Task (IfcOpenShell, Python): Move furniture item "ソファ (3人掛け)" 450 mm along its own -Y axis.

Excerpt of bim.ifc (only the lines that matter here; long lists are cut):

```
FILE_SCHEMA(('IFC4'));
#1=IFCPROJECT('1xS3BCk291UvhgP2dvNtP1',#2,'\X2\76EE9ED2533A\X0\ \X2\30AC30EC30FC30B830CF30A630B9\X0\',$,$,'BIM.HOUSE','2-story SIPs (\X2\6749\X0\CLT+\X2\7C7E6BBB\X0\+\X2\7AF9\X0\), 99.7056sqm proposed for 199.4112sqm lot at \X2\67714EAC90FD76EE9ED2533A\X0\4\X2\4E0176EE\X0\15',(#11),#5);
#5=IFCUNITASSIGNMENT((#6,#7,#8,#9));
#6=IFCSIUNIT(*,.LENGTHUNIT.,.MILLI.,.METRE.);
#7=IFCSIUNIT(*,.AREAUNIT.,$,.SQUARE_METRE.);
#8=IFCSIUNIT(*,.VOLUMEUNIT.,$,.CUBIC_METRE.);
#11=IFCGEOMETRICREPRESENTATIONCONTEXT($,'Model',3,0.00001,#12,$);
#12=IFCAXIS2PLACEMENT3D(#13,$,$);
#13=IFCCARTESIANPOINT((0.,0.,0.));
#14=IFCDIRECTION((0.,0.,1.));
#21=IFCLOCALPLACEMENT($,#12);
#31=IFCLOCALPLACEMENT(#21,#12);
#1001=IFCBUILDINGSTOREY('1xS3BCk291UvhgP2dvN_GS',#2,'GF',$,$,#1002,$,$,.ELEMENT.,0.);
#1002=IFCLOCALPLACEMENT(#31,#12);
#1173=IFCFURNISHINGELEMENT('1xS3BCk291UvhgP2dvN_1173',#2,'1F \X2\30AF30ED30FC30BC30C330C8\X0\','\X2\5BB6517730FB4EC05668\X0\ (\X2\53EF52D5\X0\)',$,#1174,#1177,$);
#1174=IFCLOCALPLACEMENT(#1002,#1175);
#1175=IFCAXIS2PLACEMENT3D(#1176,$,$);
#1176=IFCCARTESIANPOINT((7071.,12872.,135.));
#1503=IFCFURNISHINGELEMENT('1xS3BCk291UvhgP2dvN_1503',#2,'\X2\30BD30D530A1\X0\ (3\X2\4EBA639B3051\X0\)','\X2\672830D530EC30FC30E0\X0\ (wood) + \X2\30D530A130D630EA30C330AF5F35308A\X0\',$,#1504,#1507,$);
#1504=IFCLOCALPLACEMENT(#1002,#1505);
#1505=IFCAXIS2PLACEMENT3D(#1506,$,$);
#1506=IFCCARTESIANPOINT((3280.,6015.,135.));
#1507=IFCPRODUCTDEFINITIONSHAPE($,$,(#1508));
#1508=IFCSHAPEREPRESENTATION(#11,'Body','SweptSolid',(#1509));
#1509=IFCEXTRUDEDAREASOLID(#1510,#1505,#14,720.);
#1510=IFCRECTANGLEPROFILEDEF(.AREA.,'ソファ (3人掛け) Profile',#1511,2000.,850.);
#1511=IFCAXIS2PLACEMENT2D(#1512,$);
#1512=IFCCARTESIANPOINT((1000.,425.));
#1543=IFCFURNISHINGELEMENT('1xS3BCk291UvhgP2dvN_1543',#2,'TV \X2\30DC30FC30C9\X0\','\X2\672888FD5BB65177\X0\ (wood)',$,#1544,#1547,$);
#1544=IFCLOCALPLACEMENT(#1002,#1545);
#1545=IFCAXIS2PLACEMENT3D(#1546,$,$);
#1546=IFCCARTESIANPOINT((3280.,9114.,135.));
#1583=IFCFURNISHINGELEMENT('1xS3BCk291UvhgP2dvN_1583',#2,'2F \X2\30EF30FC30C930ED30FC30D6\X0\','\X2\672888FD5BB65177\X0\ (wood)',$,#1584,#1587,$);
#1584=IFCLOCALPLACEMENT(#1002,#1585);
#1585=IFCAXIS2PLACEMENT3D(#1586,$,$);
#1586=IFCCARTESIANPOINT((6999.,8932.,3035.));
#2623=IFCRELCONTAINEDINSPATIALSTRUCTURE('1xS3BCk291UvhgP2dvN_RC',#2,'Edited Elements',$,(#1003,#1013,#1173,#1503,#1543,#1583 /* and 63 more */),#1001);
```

```python
import ifcopenshell
import ifcopenshell.api.geometry
import ifcopenshell.util.placement
import ifcopenshell.util.unit

model = ifcopenshell.open("bim.ifc")
unit_scale = ifcopenshell.util.unit.calculate_unit_scale(model)

item = model.by_guid("1xS3BCk291UvhgP2dvN_1503")
matrix = ifcopenshell.util.placement.get_local_placement(item.ObjectPlacement)
matrix[:3, 3] -= matrix[:3, 1] * 0.45 / unit_scale
ifcopenshell.api.geometry.edit_object_placement(model, product=item, matrix=matrix, is_si=False)

print(ifcopenshell.util.placement.get_local_placement(item.ObjectPlacement).round(3) + 0.0)

model.write("bim_v2.ifc")
```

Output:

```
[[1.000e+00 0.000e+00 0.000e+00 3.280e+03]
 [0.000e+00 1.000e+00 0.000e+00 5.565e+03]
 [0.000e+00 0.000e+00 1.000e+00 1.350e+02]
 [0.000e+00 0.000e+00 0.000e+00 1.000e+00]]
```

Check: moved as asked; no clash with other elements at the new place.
